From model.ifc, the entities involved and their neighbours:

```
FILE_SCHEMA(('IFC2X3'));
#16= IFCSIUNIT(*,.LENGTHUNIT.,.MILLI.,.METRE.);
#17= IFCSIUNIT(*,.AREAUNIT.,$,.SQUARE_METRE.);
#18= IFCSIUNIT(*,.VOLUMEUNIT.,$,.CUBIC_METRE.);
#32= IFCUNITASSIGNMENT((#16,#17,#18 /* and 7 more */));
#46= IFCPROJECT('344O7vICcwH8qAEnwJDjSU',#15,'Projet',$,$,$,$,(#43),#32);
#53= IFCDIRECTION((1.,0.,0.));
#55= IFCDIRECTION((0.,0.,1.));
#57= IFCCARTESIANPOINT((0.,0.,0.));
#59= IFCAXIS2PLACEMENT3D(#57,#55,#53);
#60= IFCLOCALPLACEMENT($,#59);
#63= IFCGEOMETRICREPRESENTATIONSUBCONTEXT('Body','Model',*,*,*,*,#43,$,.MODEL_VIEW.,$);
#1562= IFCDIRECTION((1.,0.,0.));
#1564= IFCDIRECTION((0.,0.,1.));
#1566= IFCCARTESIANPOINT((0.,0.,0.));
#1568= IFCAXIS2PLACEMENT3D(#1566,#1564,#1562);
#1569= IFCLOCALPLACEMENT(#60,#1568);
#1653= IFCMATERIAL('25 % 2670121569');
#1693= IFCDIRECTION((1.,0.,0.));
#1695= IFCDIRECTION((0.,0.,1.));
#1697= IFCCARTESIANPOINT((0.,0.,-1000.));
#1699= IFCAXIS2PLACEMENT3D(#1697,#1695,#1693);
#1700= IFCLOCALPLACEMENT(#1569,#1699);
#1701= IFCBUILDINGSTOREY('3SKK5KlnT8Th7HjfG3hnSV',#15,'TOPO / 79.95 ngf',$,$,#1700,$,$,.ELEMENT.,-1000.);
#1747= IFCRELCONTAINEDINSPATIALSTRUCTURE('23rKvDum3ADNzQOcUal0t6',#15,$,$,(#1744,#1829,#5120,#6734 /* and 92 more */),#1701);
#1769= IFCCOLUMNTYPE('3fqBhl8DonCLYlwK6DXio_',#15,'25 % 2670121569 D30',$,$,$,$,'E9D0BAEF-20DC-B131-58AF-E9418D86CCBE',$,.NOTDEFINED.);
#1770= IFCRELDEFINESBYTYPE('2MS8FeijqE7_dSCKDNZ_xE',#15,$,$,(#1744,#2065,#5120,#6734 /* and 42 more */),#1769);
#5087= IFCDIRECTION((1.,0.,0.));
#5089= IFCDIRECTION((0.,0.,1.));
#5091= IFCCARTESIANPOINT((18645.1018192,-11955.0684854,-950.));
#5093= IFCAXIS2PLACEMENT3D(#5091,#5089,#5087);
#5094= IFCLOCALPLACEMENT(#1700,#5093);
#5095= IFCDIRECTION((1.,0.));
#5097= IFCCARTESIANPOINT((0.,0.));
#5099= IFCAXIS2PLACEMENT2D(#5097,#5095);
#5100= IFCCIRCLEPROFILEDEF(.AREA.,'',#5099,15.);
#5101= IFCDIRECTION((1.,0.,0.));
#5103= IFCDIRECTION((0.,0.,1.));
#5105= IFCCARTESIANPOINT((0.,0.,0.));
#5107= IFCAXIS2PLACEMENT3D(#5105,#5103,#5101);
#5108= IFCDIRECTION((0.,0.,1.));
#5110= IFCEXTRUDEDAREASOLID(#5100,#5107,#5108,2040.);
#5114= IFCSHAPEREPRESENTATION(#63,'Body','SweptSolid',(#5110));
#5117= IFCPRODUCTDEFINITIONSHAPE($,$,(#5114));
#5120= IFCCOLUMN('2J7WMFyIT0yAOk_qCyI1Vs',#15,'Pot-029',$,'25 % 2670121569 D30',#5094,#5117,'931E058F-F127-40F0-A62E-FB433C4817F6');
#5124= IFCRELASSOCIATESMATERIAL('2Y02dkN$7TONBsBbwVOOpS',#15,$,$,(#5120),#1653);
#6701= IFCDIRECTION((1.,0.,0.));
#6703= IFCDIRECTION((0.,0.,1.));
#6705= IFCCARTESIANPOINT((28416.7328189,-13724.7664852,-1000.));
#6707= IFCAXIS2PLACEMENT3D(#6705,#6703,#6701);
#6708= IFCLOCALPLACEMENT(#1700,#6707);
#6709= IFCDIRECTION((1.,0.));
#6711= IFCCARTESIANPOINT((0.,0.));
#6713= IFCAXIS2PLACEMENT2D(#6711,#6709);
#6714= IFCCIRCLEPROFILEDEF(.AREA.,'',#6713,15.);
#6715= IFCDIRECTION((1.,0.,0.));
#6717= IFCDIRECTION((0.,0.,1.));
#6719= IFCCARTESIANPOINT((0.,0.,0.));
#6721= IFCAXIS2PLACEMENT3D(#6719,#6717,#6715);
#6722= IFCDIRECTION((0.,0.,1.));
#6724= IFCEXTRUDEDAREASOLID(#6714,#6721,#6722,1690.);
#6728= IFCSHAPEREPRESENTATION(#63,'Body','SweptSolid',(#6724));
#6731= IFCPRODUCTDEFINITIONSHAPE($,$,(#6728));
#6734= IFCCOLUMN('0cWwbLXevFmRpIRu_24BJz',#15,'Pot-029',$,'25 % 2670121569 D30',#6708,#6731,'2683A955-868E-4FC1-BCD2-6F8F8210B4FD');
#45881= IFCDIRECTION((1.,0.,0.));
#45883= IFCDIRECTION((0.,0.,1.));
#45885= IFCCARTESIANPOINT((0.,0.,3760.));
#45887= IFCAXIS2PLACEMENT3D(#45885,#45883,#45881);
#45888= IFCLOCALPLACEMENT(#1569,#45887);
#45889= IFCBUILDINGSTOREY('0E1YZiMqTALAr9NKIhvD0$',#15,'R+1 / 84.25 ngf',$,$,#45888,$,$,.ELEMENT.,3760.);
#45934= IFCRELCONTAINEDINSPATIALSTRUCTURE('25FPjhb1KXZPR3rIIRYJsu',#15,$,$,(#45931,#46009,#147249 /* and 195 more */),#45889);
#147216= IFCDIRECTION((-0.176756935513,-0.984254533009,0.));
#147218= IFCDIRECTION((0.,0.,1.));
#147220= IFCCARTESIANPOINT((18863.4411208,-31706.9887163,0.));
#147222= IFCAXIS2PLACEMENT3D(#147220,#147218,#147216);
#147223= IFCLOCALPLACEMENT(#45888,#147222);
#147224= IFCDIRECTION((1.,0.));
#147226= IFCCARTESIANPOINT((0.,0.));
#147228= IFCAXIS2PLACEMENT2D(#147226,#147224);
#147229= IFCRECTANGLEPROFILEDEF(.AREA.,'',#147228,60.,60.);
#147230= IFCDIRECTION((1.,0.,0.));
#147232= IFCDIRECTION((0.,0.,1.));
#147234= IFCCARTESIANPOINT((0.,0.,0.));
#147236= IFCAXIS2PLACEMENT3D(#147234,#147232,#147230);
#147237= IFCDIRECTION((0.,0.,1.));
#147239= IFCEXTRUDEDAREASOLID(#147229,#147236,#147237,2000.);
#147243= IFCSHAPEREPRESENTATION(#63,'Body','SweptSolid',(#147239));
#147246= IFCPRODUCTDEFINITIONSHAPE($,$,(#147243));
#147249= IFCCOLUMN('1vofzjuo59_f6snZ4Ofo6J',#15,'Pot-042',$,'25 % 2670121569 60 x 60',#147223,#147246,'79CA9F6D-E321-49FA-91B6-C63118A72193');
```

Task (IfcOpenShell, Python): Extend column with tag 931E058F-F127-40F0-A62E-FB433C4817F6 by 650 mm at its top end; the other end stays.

```python
import ifcopenshell
import ifcopenshell.util.representation

model = ifcopenshell.open("model.ifc")

member = model.by_guid("2J7WMFyIT0yAOk_qCyI1Vs")
change = 650.0

# The extrusion runs towards the end named, so only its depth changes.
body = ifcopenshell.util.representation.get_representation(member, "Model", "Body")
solid = body.Items[0]
old_length = solid.Depth
solid.Depth += change

print(f"length {old_length:g} -> {solid.Depth:g}")

model.write("model_edited.ifc")
```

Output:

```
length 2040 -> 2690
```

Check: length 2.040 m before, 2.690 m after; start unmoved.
